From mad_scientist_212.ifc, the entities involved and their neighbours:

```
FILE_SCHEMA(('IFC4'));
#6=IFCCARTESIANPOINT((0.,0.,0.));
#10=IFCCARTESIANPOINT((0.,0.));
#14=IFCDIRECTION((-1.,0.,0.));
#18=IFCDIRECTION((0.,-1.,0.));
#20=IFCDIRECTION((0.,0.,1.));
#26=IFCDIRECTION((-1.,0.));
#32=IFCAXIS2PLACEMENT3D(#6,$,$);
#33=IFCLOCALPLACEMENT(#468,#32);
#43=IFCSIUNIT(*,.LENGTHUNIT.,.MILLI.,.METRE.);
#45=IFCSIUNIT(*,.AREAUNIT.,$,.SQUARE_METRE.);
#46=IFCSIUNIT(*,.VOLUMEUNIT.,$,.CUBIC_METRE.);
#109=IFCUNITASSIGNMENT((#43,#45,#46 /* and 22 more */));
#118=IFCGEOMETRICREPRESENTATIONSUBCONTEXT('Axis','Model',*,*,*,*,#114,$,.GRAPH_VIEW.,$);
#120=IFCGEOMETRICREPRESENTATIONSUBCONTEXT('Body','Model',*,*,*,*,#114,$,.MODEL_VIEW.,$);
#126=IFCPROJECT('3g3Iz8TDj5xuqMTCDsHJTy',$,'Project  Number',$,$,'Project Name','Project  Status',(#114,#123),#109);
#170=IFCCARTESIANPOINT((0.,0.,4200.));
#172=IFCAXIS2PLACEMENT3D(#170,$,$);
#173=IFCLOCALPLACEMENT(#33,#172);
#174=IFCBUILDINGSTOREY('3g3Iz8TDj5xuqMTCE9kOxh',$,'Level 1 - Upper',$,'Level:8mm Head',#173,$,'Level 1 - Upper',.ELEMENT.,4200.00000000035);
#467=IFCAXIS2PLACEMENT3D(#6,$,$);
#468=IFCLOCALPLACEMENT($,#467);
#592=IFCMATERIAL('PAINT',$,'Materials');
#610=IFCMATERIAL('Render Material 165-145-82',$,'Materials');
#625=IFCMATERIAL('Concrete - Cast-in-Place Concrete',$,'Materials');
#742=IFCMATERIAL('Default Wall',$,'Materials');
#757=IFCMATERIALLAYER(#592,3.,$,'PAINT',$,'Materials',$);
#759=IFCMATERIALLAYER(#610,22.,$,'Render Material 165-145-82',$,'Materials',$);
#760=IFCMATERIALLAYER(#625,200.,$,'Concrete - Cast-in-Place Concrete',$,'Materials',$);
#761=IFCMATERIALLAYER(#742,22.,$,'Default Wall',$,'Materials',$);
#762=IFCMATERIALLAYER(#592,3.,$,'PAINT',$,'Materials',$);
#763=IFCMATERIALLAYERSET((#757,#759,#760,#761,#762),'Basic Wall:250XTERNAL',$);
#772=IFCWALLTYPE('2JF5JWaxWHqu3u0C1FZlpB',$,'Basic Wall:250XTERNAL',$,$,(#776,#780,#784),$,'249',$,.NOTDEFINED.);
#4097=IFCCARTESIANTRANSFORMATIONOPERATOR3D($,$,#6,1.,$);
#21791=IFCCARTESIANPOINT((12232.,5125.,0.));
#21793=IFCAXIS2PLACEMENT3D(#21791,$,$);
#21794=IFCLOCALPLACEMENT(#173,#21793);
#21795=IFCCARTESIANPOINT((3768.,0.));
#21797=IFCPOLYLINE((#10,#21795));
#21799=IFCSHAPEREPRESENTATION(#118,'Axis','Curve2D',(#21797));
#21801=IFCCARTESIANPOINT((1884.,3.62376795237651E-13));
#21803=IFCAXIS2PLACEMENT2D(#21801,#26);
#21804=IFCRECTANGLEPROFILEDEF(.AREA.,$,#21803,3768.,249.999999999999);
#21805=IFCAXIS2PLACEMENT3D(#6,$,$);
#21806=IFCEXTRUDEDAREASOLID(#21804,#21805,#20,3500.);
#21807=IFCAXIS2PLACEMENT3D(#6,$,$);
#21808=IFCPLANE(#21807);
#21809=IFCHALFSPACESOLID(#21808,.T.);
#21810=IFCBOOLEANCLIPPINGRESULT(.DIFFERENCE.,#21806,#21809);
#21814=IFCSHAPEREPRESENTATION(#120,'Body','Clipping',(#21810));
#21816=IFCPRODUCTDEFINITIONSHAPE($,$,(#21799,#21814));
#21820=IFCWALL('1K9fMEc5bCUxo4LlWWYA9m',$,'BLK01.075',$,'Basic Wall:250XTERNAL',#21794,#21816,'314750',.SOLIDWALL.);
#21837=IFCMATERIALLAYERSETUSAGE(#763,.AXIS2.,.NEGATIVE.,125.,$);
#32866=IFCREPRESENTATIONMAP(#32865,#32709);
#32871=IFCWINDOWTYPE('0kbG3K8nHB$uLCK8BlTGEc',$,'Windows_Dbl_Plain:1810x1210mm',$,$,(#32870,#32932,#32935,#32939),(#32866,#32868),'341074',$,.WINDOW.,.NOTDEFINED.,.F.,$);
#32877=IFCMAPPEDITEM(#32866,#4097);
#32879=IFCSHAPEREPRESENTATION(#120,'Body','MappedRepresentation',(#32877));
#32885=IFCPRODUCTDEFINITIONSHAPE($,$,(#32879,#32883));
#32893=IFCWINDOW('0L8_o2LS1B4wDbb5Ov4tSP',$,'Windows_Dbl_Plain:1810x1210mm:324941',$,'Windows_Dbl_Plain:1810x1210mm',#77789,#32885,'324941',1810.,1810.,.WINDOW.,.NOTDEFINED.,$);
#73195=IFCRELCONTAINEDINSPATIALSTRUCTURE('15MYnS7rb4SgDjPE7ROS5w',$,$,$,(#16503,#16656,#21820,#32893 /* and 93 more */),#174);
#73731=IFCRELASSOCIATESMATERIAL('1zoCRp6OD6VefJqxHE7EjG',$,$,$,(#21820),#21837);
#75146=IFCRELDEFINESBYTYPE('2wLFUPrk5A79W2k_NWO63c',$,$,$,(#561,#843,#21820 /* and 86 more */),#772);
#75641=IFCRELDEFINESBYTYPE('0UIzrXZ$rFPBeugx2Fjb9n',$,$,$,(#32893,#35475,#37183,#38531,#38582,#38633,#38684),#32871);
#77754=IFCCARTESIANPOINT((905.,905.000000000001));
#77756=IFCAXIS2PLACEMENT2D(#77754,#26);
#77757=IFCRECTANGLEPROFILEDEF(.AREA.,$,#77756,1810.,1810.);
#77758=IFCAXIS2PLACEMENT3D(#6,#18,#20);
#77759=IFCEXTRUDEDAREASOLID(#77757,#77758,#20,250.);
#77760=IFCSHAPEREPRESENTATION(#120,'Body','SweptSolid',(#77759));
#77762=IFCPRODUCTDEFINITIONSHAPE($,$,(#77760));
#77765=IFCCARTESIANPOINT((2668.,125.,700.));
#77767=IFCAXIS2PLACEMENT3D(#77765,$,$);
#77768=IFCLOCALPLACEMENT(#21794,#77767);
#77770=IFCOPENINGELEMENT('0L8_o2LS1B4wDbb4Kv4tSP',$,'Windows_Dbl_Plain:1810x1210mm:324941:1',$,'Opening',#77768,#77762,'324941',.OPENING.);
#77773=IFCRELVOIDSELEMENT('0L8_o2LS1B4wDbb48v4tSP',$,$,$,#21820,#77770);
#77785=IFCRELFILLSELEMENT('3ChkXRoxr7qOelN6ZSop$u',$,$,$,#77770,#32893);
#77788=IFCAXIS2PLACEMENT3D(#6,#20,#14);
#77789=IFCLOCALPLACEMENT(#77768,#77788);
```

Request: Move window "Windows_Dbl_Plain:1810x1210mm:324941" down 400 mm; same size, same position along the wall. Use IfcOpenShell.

```python
import numpy as np
import ifcopenshell
import ifcopenshell.api.geometry
import ifcopenshell.util.placement
import ifcopenshell.util.unit

model = ifcopenshell.open("mad_scientist_212.ifc")
unit_scale = ifcopenshell.util.unit.calculate_unit_scale(model)

window = model.by_guid("0L8_o2LS1B4wDbb5Ov4tSP")
opening = window.FillsVoids[0].RelatingOpeningElement
dz = -400.0

shift = np.array([0.0, 0.0, dz])
# The window is placed relative to its opening, so it follows when the opening moves.
matrix = ifcopenshell.util.placement.get_local_placement(opening.ObjectPlacement)
matrix[:3, 3] += shift
ifcopenshell.api.geometry.edit_object_placement(
    model, product=opening, matrix=matrix, is_si=False, should_transform_children=True
)

print(f"moved by {dz * unit_scale:+.3f} m")

model.write("mad_scientist_212_rev.ifc")
```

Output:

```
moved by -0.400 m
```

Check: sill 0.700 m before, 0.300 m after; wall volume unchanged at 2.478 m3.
